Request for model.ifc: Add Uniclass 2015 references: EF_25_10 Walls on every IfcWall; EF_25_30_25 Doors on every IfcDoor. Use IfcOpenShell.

First a look at what the model holds.

```python
import ifcopenshell

model = ifcopenshell.open("model.ifc")
print(model.schema)
print("classifications:", [c.Name for c in model.by_type("IfcClassification")])
for ifc_class in ("IfcDoor", "IfcRoof", "IfcStair", "IfcWall", "IfcWindow"):
    print(ifc_class, len(model.by_type(ifc_class)))
```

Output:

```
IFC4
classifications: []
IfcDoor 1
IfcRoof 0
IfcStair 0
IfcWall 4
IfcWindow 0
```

```python
import ifcopenshell
import ifcopenshell.api.classification

model = ifcopenshell.open("model.ifc")

system = ifcopenshell.api.classification.add_classification(model, classification="Uniclass 2015")

codes = {
    "IfcWall": ("EF_25_10", "Walls"),
    "IfcDoor": ("EF_25_30_25", "Doors"),
}
for ifc_class, (code, name) in codes.items():
    products = model.by_type(ifc_class)
    ifcopenshell.api.classification.add_reference(
        model, products=products, classification=system, identification=code, name=name
    )
    print(code, len(products))

model.write("model-out.ifc")
```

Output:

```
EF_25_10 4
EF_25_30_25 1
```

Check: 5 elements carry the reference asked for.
